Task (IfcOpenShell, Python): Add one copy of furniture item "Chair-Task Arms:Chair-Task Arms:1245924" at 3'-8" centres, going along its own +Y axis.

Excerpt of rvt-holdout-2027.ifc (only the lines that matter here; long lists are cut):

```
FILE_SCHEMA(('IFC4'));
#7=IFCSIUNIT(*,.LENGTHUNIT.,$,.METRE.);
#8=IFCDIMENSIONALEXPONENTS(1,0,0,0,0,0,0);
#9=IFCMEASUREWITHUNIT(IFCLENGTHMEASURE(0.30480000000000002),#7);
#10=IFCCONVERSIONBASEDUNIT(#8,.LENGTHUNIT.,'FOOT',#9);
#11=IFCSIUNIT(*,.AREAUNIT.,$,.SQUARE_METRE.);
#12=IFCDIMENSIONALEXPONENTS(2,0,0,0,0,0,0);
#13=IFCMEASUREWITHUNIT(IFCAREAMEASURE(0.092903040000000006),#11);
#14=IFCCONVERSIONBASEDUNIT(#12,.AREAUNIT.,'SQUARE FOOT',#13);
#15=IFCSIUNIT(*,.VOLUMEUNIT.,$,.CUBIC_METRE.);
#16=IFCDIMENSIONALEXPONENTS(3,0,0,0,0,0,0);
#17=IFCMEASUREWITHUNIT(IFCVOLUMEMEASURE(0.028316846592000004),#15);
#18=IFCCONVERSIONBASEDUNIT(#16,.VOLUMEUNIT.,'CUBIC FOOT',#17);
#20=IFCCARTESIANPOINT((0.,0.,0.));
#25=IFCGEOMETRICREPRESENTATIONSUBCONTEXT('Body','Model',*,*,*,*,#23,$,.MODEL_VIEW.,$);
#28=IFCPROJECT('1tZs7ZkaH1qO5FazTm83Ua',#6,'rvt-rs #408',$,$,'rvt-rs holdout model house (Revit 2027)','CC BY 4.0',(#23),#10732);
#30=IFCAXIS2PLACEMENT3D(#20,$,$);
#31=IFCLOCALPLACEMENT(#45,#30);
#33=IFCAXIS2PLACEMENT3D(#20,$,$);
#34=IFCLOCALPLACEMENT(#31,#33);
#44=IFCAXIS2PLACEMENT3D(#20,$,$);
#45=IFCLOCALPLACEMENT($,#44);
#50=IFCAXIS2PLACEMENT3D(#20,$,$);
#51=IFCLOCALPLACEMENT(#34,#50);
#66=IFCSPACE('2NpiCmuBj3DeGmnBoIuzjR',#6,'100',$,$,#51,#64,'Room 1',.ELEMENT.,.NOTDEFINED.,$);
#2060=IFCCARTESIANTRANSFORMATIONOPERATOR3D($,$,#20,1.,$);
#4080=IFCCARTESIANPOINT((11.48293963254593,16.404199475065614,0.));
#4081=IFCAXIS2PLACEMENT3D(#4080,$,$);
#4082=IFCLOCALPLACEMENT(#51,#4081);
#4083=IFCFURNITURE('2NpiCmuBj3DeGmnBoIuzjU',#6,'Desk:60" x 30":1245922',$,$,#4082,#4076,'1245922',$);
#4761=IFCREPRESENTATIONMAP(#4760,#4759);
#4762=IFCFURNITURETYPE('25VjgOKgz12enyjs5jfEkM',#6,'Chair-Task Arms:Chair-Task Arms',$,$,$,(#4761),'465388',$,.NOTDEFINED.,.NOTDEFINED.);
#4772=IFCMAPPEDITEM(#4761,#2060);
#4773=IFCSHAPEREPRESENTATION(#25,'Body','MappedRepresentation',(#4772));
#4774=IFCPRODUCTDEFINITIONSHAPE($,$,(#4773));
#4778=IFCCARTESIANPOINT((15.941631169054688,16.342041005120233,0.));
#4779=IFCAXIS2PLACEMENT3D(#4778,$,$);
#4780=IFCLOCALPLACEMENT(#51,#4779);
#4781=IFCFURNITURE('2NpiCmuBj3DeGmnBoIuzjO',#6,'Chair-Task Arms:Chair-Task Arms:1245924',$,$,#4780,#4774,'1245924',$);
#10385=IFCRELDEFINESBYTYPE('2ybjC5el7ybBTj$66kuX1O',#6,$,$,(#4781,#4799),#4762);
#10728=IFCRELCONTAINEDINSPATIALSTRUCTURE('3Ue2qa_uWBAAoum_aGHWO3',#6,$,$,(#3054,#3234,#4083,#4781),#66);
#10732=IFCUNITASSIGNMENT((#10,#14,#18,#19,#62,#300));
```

```python
import ifcopenshell
import ifcopenshell.api.geometry
import ifcopenshell.api.root
import ifcopenshell.util.element
import ifcopenshell.util.placement
import ifcopenshell.util.unit

model = ifcopenshell.open("rvt-holdout-2027.ifc")
unit_scale = ifcopenshell.util.unit.calculate_unit_scale(model)


def reuse_history(source, copy):
    """copy_class also copies each property set's owner history, people and application; keep the originals."""
    for rel in copy.IsDefinedBy:
        if rel.is_a("IfcRelDefinesByProperties") and (history := rel.RelatingPropertyDefinition.OwnerHistory):
            rel.RelatingPropertyDefinition.OwnerHistory = source.OwnerHistory
            ifcopenshell.util.element.remove_deep2(model, history)


source = model.by_guid("2NpiCmuBj3DeGmnBoIuzjO")
base = ifcopenshell.util.placement.get_local_placement(source.ObjectPlacement)
step = base[:3, 1] * 44 * 0.0254 / unit_scale

for i in range(1, 2):
    copy = ifcopenshell.api.root.copy_class(model, product=source)
    copy.Representation = ifcopenshell.util.element.copy_deep(
        model, source.Representation, exclude=["IfcGeometricRepresentationContext", "IfcRepresentationMap"]
    )
    copy.Name = "Chair-Task Arms:Chair-Task Arms"
    copy.Tag = None
    reuse_history(source, copy)
    matrix = base.copy()
    matrix[:3, 3] += i * step
    print("added at", matrix[:3, 3].round(3) + 0.0)
    ifcopenshell.api.geometry.edit_object_placement(model, product=copy, matrix=matrix, is_si=False)

model.write("rvt-holdout-2027_updated.ifc")
```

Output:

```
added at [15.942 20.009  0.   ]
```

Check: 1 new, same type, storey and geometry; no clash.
